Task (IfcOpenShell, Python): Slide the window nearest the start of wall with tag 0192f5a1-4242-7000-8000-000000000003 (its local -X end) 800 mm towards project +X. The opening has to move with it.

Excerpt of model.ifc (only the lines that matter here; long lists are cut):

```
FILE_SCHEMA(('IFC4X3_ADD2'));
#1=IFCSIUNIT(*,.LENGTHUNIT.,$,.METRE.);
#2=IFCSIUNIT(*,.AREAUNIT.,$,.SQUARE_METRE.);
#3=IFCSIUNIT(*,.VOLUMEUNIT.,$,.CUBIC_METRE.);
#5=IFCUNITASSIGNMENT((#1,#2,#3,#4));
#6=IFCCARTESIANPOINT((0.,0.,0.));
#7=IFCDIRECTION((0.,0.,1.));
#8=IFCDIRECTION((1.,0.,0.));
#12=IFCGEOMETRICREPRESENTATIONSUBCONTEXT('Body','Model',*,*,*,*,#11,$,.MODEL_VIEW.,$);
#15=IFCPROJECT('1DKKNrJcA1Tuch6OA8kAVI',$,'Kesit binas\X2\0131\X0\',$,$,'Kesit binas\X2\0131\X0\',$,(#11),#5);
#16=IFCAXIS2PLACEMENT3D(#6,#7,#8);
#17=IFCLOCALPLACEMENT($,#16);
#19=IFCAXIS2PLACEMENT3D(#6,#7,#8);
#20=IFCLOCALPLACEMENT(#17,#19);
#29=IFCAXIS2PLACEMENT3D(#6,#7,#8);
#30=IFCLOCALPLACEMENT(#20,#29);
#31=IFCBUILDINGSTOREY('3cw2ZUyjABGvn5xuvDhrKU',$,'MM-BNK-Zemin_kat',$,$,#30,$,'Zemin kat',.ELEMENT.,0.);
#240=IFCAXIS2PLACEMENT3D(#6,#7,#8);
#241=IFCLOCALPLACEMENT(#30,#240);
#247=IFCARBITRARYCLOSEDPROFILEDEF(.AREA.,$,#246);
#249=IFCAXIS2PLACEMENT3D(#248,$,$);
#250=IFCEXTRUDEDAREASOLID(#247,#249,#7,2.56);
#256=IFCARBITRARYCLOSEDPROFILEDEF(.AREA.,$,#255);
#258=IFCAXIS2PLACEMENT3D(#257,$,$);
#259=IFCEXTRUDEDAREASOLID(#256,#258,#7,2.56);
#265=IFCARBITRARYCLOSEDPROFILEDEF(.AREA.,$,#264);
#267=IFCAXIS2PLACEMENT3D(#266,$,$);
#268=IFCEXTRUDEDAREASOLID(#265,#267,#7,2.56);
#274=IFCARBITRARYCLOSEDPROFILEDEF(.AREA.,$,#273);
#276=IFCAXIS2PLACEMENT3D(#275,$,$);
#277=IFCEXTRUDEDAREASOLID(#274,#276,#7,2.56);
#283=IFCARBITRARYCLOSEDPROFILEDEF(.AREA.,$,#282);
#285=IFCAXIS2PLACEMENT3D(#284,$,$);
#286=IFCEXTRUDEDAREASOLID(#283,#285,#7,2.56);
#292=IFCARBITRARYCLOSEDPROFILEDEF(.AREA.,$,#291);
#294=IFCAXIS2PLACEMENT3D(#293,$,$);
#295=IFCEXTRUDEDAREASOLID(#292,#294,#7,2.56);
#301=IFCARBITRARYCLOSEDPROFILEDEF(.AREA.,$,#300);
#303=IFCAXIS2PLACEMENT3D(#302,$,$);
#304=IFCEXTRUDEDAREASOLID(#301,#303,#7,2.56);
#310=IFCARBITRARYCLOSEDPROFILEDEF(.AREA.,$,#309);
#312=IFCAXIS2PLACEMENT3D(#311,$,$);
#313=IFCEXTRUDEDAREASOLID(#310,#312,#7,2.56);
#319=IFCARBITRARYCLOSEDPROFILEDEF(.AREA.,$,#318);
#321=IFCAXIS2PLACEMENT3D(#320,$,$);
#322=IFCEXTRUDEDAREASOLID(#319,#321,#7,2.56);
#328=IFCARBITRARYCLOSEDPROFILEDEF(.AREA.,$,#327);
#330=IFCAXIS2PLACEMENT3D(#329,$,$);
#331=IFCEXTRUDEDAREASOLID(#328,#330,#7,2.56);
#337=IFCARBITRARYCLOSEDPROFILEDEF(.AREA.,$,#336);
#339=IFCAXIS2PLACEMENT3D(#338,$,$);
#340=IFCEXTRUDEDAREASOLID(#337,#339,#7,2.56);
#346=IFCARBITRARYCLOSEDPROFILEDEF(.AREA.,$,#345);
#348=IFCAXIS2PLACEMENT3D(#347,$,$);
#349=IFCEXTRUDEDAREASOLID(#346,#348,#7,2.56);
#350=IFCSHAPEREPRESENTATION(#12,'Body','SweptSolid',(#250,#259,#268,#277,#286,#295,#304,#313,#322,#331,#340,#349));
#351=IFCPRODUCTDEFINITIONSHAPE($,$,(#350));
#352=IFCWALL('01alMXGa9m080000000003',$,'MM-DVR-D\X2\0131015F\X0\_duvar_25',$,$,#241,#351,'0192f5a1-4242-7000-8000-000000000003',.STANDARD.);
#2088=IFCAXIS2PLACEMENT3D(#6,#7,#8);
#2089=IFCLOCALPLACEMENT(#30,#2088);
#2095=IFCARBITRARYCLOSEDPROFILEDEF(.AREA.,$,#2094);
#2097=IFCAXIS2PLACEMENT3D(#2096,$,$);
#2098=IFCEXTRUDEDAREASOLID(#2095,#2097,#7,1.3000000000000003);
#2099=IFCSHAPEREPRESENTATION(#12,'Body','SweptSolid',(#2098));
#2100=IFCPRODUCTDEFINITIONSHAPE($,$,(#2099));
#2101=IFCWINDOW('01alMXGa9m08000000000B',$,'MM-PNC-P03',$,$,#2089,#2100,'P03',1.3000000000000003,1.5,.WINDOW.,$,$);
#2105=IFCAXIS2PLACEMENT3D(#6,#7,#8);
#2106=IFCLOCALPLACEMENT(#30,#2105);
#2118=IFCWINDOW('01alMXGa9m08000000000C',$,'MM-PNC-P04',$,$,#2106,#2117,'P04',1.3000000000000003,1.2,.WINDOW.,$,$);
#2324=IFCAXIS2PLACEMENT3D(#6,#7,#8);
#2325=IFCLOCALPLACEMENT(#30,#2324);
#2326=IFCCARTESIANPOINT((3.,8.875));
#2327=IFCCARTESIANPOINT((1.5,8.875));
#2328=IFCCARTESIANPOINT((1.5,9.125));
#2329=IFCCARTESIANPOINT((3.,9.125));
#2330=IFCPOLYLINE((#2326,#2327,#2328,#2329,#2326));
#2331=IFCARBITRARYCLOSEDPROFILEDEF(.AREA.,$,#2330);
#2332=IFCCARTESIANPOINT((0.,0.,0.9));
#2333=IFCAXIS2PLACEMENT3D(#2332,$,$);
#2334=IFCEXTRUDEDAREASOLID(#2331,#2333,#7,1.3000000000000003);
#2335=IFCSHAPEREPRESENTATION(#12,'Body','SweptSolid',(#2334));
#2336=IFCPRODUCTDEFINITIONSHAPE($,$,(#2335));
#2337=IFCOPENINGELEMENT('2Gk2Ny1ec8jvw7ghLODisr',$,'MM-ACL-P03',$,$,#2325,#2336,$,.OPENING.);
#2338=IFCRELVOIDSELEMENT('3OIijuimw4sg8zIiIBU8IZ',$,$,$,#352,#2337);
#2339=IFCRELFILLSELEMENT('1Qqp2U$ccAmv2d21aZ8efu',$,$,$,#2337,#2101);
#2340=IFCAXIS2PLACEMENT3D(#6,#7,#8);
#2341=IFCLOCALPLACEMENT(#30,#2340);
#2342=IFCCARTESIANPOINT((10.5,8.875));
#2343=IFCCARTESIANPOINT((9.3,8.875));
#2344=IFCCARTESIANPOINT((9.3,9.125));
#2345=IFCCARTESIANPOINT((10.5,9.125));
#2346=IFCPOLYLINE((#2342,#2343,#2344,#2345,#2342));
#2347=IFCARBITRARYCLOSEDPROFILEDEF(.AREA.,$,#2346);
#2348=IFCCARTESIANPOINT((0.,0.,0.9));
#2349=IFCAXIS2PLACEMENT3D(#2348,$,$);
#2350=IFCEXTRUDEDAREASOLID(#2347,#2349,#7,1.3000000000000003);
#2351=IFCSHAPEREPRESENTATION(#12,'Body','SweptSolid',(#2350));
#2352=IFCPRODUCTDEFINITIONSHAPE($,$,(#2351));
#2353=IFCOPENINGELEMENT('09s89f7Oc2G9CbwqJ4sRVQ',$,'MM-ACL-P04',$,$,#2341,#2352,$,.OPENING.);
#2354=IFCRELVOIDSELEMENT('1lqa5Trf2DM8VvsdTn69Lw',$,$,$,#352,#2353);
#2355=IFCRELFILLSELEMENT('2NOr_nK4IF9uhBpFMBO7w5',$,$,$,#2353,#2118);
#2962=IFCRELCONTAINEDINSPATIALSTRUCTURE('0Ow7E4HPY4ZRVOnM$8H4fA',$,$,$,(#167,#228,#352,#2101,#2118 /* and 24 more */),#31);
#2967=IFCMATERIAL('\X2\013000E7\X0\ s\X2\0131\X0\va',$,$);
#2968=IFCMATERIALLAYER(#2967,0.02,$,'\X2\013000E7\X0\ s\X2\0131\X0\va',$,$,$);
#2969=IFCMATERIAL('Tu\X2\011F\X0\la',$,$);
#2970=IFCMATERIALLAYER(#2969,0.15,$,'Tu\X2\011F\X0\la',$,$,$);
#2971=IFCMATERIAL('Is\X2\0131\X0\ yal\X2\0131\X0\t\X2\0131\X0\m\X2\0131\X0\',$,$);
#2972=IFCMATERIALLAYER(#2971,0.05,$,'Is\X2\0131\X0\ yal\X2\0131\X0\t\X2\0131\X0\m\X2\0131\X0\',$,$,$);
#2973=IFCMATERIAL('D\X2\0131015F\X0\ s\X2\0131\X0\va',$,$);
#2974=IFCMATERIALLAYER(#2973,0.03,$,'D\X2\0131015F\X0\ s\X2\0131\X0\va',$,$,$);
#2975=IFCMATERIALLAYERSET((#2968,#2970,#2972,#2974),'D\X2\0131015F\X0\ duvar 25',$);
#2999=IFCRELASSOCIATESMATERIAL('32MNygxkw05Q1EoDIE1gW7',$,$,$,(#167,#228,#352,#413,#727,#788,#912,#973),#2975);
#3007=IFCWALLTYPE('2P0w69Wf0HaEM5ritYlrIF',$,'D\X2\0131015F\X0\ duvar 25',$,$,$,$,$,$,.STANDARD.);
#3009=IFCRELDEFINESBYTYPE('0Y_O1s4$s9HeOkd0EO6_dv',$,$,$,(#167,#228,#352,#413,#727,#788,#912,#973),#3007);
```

```python
import ifcopenshell
import ifcopenshell.api.geometry
import ifcopenshell.util.placement
import ifcopenshell.util.unit

model = ifcopenshell.open("model.ifc")
unit_scale = ifcopenshell.util.unit.calculate_unit_scale(model)

window = model.by_guid("01alMXGa9m08000000000B")
opening = window.FillsVoids[0].RelatingOpeningElement
wall = opening.VoidsElements[0].RelatingBuildingElement

wall_matrix = ifcopenshell.util.placement.get_local_placement(wall.ObjectPlacement)
shift = wall_matrix[:3, 0] * 0.8 / unit_scale
before = ifcopenshell.util.placement.get_local_placement(window.ObjectPlacement)[:3, 3].copy()

# The window is not placed relative to its opening, so move both.
for product in (opening, window):
    matrix = ifcopenshell.util.placement.get_local_placement(product.ObjectPlacement)
    matrix[:3, 3] += shift
    ifcopenshell.api.geometry.edit_object_placement(model, product=product, matrix=matrix, is_si=False)

after = ifcopenshell.util.placement.get_local_placement(window.ObjectPlacement)[:3, 3]
print("window moved by", (after - before).round(3) + 0.0)

model.write("model_edited.ifc")
```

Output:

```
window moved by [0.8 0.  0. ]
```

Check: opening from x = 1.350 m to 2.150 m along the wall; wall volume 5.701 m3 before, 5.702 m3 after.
